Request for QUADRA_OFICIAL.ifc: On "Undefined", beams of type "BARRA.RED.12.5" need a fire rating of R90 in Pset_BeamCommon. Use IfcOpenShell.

First a look at what the model holds.

```python
import ifcopenshell
import ifcopenshell.util.element

model = ifcopenshell.open("QUADRA_OFICIAL.ifc")
print(model.schema)
storey = next(s for s in model.by_type("IfcBuildingStorey") if s.Name == "Undefined")
beams = [e for e in ifcopenshell.util.element.get_decomposition(storey) if e.is_a("IfcBeam")]
seen = {}
for e in beams:
    element_type = ifcopenshell.util.element.get_type(e)
    key = (element_type.Name if element_type != e and element_type else None, ifcopenshell.util.element.get_pset(e, "Pset_BeamCommon", "FireRating"))
    seen[key] = seen.get(key, 0) + 1
for (name, value), count in sorted(seen.items(), key=str):
    print(count, "x", name, "|", value)
```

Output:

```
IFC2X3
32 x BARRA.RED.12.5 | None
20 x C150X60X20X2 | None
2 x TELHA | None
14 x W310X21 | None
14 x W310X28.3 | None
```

```python
import ifcopenshell
import ifcopenshell.api.pset
import ifcopenshell.util.element

model = ifcopenshell.open("QUADRA_OFICIAL.ifc")

storey = next(s for s in model.by_type("IfcBuildingStorey") if s.Name == "Undefined")
beams = [e for e in ifcopenshell.util.element.get_decomposition(storey) if e.is_a("IfcBeam")]

count = 0
for e in beams:
    element_type = ifcopenshell.util.element.get_type(e)
    if element_type in (None, e) or element_type.Name != "BARRA.RED.12.5":
        continue
    found = ifcopenshell.util.element.get_pset(e, "Pset_BeamCommon", should_inherit=False)
    if found:
        pset = model.by_id(found["id"])
        if len(ifcopenshell.util.element.get_elements_by_pset(pset)) > 1:
            pset = ifcopenshell.api.pset.unshare_pset(model, products=[e], pset=pset)[0]
    else:
        pset = ifcopenshell.api.pset.add_pset(model, product=e, name="Pset_BeamCommon")
    ifcopenshell.api.pset.edit_pset(model, pset=pset, properties={"FireRating": "R90"})
    count += 1

print(count, "beams updated")

model.write("QUADRA_OFICIAL_v2.ifc")
```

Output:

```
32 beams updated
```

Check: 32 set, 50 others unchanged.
